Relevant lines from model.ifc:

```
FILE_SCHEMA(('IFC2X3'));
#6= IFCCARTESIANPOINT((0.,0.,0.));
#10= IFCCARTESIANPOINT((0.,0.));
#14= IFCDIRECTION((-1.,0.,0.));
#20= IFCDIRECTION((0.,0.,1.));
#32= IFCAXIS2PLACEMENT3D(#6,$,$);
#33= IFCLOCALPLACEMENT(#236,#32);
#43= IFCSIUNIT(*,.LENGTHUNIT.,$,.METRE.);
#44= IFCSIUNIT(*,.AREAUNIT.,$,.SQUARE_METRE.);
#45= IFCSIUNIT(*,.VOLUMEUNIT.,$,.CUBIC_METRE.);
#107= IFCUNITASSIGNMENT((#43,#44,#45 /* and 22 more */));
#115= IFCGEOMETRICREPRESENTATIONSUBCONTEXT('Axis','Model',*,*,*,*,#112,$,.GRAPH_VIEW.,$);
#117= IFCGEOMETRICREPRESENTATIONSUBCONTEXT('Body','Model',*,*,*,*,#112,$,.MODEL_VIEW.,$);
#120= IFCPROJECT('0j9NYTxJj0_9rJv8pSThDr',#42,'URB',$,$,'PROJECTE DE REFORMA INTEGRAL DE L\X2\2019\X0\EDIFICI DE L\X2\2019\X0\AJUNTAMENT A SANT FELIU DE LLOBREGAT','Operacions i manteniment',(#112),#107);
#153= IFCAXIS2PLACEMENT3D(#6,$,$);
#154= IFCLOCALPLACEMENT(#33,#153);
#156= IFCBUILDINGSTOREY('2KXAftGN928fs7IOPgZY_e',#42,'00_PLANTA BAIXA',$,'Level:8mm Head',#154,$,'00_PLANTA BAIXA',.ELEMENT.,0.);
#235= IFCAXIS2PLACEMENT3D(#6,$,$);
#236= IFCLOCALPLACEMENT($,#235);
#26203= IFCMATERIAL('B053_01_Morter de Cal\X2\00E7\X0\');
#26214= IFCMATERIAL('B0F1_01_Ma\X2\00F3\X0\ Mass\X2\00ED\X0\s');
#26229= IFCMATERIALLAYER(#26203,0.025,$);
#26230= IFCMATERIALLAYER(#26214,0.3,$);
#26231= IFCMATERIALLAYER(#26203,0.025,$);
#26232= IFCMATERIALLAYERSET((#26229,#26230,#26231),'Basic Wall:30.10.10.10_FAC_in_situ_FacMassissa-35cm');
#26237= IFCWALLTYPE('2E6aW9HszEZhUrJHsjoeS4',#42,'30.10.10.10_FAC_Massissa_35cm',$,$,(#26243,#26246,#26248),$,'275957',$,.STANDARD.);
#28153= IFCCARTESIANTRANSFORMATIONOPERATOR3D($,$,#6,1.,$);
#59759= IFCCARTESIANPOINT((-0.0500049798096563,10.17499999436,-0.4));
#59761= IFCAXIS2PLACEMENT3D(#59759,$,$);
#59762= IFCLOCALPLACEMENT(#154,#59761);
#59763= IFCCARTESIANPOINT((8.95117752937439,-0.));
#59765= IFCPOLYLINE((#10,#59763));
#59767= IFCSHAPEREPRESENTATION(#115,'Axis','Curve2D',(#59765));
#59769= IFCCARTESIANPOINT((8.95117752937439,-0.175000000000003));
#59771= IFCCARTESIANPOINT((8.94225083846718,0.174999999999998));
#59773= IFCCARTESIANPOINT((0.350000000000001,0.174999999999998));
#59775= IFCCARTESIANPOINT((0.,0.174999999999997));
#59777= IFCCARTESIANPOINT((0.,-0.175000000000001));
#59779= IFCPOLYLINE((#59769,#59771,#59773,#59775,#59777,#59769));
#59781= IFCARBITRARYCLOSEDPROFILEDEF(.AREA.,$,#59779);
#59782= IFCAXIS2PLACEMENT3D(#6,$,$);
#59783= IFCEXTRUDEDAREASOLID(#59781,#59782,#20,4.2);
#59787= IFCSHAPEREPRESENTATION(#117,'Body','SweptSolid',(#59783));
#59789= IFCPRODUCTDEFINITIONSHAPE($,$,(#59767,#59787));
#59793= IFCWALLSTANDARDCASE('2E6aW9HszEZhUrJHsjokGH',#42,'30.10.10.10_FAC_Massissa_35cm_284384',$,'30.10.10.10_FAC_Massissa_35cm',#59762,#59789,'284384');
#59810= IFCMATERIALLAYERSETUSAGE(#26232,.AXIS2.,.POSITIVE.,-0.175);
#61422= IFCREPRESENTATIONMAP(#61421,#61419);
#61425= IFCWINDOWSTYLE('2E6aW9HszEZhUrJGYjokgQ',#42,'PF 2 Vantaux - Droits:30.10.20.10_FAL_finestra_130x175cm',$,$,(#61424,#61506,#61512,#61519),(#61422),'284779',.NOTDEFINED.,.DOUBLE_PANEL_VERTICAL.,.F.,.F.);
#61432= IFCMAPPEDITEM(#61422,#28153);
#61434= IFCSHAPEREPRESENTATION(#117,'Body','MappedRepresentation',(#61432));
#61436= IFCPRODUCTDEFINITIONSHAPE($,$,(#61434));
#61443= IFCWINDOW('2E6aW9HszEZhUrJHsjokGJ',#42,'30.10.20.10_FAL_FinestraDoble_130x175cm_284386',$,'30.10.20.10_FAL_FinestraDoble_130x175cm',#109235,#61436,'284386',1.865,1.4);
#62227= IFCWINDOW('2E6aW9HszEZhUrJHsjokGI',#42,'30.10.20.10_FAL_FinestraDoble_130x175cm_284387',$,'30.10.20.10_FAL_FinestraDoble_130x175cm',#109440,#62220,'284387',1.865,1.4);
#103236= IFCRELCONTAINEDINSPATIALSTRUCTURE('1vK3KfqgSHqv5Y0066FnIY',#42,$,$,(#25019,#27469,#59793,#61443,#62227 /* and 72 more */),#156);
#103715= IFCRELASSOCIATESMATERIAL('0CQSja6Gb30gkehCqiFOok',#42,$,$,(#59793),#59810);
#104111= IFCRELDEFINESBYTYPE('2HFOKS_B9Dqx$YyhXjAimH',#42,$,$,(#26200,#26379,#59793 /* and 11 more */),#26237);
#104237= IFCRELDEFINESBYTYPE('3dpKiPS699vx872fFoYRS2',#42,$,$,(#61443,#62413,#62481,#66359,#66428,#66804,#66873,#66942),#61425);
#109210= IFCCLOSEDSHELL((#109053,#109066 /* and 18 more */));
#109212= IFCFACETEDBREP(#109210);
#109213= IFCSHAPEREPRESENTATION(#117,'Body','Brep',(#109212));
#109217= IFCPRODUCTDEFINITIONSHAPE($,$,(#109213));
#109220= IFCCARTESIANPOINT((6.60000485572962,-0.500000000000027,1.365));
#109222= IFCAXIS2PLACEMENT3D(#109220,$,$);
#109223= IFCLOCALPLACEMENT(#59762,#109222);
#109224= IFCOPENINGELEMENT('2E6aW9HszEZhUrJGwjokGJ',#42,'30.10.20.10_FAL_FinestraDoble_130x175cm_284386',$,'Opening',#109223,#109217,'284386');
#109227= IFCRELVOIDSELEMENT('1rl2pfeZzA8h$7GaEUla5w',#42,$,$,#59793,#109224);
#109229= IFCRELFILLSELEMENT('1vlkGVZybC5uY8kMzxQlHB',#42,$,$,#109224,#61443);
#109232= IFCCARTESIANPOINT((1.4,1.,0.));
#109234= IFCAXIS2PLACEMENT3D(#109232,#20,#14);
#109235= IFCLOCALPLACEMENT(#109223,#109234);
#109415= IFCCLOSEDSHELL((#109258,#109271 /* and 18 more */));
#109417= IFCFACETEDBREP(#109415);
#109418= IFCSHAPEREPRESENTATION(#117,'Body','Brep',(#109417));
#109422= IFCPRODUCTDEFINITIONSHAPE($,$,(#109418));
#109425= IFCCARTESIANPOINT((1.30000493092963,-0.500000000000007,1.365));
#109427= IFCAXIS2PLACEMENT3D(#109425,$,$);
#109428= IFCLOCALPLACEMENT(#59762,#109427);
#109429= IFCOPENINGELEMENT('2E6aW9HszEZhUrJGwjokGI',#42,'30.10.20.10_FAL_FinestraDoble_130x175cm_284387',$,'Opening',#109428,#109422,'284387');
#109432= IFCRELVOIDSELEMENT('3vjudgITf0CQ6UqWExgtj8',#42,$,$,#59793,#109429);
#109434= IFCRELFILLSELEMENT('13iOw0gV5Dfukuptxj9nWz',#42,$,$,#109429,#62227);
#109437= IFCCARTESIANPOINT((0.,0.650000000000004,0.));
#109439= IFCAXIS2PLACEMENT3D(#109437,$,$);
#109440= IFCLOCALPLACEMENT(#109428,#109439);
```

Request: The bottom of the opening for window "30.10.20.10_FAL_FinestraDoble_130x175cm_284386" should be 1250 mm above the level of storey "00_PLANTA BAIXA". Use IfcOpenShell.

```python
import numpy as np
import ifcopenshell
import ifcopenshell.api.geometry
import ifcopenshell.geom
import ifcopenshell.util.element
import ifcopenshell.util.placement
import ifcopenshell.util.shape
import ifcopenshell.util.unit

model = ifcopenshell.open("model.ifc")
unit_scale = ifcopenshell.util.unit.calculate_unit_scale(model)

window = model.by_guid("2E6aW9HszEZhUrJHsjokGJ")
opening = window.FillsVoids[0].RelatingOpeningElement
storey = ifcopenshell.util.element.get_container(window, ifc_class="IfcBuildingStorey")
level = ifcopenshell.util.placement.get_local_placement(storey.ObjectPlacement)[2, 3]

# The opening's origin need not be at the sill, so measure its lowest point.
shape = ifcopenshell.geom.create_shape(ifcopenshell.geom.settings(), opening)
bottom = ifcopenshell.util.shape.get_shape_bottom_elevation(shape, shape.geometry) / unit_scale
dz = level + 1.25 - bottom

shift = np.array([0.0, 0.0, dz])
# The window is placed relative to its opening, so it follows when the opening moves.
matrix = ifcopenshell.util.placement.get_local_placement(opening.ObjectPlacement)
matrix[:3, 3] += shift
ifcopenshell.api.geometry.edit_object_placement(
    model, product=opening, matrix=matrix, is_si=False, should_transform_children=True
)

print(f"moved by {dz * unit_scale:+.3f} m")

model.write("model-out.ifc")
```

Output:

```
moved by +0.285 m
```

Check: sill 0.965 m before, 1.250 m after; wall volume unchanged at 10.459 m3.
